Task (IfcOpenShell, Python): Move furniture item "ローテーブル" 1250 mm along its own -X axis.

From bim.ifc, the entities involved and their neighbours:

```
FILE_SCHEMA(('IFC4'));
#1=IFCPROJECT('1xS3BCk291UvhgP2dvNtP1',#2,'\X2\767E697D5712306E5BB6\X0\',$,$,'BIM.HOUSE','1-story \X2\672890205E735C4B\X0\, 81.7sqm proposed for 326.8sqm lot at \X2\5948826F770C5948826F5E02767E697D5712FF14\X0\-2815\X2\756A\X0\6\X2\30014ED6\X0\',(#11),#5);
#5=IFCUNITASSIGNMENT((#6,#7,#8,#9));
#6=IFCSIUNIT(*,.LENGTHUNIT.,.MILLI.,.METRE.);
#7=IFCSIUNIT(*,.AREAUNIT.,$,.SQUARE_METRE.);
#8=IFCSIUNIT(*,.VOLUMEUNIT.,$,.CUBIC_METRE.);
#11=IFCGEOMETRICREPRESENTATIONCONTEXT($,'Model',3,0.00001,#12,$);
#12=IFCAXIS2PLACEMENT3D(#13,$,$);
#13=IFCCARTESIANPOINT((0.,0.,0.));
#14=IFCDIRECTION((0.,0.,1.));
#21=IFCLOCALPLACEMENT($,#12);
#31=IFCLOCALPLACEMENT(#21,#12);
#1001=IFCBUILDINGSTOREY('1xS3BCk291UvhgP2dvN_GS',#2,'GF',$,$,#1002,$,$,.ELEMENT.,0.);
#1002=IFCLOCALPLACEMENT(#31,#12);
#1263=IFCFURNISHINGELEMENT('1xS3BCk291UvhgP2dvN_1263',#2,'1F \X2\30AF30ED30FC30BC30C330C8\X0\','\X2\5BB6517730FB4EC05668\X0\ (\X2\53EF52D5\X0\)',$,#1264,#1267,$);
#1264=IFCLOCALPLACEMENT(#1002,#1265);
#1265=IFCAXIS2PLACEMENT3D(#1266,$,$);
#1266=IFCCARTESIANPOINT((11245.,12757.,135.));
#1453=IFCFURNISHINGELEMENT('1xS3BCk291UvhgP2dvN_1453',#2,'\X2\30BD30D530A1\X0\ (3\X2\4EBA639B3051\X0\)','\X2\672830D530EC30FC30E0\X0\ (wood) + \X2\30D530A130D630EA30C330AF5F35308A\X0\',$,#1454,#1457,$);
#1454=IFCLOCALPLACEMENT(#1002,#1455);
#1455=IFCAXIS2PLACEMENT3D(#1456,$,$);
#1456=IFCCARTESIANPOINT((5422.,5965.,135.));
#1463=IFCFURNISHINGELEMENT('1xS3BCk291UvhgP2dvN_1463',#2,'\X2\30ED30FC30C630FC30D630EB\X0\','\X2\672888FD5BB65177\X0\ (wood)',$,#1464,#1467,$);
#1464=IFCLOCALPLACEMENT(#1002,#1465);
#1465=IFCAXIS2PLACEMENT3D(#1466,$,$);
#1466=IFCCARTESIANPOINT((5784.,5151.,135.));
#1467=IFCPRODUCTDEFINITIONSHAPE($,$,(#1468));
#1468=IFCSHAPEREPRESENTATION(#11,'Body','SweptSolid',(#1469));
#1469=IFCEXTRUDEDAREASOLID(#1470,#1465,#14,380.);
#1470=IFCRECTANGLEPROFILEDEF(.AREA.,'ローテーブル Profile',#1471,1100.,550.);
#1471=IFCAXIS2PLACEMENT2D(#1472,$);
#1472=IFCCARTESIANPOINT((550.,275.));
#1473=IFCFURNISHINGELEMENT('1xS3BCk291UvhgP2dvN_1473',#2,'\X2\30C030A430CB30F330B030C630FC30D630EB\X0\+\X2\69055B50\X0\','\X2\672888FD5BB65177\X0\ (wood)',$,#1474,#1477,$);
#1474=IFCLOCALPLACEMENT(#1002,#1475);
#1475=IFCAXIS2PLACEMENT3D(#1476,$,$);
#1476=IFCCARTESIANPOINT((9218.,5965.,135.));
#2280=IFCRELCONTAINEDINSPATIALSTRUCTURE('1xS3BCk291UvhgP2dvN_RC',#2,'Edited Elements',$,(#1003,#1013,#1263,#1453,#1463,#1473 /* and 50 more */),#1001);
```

```python
import ifcopenshell
import ifcopenshell.api.geometry
import ifcopenshell.util.placement
import ifcopenshell.util.unit

model = ifcopenshell.open("bim.ifc")
unit_scale = ifcopenshell.util.unit.calculate_unit_scale(model)

item = model.by_guid("1xS3BCk291UvhgP2dvN_1463")
matrix = ifcopenshell.util.placement.get_local_placement(item.ObjectPlacement)
matrix[:3, 3] -= matrix[:3, 0] * 1.25 / unit_scale
ifcopenshell.api.geometry.edit_object_placement(model, product=item, matrix=matrix, is_si=False)

print(ifcopenshell.util.placement.get_local_placement(item.ObjectPlacement).round(3) + 0.0)

model.write("bim_rev.ifc")
```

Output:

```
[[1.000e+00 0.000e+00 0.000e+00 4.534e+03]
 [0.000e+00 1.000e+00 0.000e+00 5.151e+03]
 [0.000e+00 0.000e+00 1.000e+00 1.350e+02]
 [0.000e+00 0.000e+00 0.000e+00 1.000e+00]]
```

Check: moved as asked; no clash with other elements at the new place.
